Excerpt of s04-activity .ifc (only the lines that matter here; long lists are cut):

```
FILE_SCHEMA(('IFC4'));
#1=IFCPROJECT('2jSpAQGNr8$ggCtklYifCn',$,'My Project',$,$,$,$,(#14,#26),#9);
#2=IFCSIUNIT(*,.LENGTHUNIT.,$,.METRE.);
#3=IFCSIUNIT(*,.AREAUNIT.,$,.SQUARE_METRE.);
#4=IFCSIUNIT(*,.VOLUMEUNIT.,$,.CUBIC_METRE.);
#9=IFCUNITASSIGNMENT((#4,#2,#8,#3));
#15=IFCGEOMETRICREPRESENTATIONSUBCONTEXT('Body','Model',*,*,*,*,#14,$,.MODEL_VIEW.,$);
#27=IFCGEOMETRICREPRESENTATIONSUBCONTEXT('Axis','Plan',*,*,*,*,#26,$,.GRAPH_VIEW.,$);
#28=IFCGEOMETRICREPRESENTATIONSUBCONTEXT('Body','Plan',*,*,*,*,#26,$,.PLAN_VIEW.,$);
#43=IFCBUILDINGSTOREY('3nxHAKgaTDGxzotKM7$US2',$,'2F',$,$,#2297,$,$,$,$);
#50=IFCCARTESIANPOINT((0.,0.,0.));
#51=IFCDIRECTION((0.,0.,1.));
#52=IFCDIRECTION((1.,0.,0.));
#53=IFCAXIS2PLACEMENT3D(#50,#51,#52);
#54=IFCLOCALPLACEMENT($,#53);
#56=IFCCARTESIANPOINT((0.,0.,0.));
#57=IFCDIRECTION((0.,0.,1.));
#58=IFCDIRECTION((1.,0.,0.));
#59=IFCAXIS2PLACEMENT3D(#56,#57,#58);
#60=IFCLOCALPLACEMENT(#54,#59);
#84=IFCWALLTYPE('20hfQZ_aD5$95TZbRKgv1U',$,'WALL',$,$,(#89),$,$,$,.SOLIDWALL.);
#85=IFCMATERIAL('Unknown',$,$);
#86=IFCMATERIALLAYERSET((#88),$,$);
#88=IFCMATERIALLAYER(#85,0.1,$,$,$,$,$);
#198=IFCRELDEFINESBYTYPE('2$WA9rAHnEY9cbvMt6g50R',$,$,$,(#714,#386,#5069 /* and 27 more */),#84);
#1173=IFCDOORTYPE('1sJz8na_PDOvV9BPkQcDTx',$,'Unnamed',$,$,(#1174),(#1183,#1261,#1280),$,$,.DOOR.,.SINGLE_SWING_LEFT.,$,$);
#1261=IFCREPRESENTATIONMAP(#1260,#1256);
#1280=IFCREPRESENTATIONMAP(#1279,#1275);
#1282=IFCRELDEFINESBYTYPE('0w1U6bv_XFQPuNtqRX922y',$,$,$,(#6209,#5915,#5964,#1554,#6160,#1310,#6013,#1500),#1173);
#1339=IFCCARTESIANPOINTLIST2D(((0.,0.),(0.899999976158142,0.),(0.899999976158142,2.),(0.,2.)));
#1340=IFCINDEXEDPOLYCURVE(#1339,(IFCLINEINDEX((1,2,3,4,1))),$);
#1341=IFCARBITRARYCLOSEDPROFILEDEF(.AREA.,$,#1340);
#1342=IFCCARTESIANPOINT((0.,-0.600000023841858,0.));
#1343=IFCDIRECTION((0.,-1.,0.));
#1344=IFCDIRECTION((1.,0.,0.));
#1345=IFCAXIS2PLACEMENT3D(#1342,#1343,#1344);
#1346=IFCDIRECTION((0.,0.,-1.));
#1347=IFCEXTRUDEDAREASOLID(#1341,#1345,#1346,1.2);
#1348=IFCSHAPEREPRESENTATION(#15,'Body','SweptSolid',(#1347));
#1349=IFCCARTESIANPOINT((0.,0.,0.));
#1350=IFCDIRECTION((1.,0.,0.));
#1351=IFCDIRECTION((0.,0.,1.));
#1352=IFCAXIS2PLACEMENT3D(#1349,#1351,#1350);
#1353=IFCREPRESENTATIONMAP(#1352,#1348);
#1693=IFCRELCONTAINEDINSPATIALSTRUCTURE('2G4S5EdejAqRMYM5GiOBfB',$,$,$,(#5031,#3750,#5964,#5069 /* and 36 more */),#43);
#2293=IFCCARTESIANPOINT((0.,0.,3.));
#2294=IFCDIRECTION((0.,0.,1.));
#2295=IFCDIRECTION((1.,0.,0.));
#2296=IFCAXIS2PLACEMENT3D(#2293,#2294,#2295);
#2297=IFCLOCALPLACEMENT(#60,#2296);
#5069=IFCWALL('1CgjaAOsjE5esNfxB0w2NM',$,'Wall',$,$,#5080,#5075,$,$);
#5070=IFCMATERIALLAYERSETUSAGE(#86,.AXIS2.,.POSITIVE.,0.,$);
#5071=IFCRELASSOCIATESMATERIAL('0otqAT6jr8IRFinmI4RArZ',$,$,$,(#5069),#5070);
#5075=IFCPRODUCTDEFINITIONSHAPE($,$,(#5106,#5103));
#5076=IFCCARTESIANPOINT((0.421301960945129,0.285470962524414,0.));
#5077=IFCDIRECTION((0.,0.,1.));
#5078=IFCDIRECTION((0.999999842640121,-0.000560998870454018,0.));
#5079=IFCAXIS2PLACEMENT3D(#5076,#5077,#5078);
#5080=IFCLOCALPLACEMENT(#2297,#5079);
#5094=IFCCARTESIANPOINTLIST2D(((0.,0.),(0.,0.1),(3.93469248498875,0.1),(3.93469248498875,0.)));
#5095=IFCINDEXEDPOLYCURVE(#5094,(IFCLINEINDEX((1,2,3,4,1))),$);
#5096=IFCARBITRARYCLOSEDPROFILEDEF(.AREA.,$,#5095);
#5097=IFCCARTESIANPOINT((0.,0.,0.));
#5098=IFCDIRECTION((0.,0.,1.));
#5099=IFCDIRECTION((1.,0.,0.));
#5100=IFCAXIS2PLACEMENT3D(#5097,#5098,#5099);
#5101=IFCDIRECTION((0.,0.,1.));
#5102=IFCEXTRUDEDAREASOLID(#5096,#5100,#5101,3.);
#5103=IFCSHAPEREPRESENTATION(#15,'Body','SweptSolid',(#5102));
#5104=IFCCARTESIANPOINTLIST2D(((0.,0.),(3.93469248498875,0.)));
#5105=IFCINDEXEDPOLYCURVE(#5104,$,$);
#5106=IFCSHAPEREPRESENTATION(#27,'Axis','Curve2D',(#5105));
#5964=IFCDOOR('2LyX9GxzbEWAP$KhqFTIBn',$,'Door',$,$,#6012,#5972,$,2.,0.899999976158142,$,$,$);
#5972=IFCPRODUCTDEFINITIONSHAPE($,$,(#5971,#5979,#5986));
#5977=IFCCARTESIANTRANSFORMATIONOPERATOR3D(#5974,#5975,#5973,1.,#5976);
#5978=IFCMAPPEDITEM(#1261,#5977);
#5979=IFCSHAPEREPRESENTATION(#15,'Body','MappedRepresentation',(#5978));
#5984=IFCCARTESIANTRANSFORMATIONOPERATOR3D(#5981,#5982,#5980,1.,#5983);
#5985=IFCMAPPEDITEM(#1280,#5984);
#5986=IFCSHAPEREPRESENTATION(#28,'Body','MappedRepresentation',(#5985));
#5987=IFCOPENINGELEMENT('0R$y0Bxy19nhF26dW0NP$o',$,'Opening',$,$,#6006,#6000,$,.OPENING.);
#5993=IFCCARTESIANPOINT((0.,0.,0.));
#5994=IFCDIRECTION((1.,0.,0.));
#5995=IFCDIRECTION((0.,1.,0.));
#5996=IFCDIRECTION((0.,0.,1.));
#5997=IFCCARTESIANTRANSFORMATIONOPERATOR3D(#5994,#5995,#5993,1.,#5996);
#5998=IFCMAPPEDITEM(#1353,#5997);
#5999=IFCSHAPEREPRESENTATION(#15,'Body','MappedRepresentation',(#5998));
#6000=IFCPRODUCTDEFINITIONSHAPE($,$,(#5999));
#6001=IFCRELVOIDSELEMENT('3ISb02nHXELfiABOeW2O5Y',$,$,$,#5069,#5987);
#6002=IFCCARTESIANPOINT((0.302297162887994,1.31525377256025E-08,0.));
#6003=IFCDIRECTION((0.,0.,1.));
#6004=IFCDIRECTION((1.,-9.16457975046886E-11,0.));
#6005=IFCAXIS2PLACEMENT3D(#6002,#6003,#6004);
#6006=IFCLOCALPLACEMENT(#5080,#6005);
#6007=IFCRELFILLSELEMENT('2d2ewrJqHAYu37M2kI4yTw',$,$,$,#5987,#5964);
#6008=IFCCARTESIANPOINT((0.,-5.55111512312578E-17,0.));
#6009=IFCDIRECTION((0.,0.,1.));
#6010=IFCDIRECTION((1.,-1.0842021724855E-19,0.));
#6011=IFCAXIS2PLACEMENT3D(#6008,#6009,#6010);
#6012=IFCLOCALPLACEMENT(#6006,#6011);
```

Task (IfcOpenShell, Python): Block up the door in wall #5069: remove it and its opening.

```python
import ifcopenshell
import ifcopenshell.api.feature
import ifcopenshell.api.root
import ifcopenshell.geom
import ifcopenshell.util.shape

model = ifcopenshell.open("s04-activity .ifc")
settings = ifcopenshell.geom.settings()


def volume(element):
    """Net volume in cubic metres, openings subtracted."""
    shape = ifcopenshell.geom.create_shape(settings, element)
    return ifcopenshell.util.shape.get_volume(shape.geometry)


door = model.by_guid("2LyX9GxzbEWAP$KhqFTIBn")
opening = door.FillsVoids[0].RelatingOpeningElement
wall = opening.VoidsElements[0].RelatingBuildingElement
before = volume(wall)

ifcopenshell.api.root.remove_product(model, product=door)
ifcopenshell.api.feature.remove_feature(model, feature=opening)

after = volume(wall)

print(f"wall volume {before:.3f} -> {after:.3f} m3")

model.write("s04-activity -out.ifc")
```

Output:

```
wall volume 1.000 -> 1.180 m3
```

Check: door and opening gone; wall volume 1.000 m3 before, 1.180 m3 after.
